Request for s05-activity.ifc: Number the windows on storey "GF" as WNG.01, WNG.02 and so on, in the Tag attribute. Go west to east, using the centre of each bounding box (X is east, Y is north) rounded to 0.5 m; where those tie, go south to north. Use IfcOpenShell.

First a look at what the model holds.

```python
import ifcopenshell
import ifcopenshell.util.element
import ifcopenshell.util.placement

model = ifcopenshell.open("s05-activity.ifc")
print(model.schema)
storey = next(s for s in model.by_type("IfcBuildingStorey") if s.Name == "GF")
windows = [e for e in ifcopenshell.util.element.get_decomposition(storey) if e.is_a("IfcWindow")]
for e in sorted(windows, key=lambda e: e.id()):
    origin = ifcopenshell.util.placement.get_local_placement(e.ObjectPlacement)[:3, 3]
    print(e.id(), e.Tag, e.Name, origin.round(2) + 0.0, sep=" | ")
```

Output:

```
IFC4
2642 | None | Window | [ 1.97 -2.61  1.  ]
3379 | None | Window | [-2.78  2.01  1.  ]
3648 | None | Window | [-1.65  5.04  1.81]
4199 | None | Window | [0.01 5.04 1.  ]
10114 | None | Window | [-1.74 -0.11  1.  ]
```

```python
import ifcopenshell
import ifcopenshell.geom
import ifcopenshell.util.element
import ifcopenshell.util.shape

model = ifcopenshell.open("s05-activity.ifc")
settings = ifcopenshell.geom.settings()
settings.set("use-world-coords", True)


def centre(element):
    shape = ifcopenshell.geom.create_shape(settings, element)
    return ifcopenshell.util.shape.get_bbox_centroid(shape.geometry)


storey = next(s for s in model.by_type("IfcBuildingStorey") if s.Name == "GF")
windows = [e for e in ifcopenshell.util.element.get_decomposition(storey) if e.is_a("IfcWindow")]

# Insertion points can sit at a corner or the storey origin, so sort by the geometry (in metres).
centres = {e: centre(e) for e in windows}
windows.sort(key=lambda e: (round(centres[e][0] / 0.5), centres[e][1]))

for i, e in enumerate(windows, start=1):
    number = f"WNG.{i:02d}"
    e.Tag = number
    print(e.id(), number)

model.write("s05-activity_edited.ifc")
```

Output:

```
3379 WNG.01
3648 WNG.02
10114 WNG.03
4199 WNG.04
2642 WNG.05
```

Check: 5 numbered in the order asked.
